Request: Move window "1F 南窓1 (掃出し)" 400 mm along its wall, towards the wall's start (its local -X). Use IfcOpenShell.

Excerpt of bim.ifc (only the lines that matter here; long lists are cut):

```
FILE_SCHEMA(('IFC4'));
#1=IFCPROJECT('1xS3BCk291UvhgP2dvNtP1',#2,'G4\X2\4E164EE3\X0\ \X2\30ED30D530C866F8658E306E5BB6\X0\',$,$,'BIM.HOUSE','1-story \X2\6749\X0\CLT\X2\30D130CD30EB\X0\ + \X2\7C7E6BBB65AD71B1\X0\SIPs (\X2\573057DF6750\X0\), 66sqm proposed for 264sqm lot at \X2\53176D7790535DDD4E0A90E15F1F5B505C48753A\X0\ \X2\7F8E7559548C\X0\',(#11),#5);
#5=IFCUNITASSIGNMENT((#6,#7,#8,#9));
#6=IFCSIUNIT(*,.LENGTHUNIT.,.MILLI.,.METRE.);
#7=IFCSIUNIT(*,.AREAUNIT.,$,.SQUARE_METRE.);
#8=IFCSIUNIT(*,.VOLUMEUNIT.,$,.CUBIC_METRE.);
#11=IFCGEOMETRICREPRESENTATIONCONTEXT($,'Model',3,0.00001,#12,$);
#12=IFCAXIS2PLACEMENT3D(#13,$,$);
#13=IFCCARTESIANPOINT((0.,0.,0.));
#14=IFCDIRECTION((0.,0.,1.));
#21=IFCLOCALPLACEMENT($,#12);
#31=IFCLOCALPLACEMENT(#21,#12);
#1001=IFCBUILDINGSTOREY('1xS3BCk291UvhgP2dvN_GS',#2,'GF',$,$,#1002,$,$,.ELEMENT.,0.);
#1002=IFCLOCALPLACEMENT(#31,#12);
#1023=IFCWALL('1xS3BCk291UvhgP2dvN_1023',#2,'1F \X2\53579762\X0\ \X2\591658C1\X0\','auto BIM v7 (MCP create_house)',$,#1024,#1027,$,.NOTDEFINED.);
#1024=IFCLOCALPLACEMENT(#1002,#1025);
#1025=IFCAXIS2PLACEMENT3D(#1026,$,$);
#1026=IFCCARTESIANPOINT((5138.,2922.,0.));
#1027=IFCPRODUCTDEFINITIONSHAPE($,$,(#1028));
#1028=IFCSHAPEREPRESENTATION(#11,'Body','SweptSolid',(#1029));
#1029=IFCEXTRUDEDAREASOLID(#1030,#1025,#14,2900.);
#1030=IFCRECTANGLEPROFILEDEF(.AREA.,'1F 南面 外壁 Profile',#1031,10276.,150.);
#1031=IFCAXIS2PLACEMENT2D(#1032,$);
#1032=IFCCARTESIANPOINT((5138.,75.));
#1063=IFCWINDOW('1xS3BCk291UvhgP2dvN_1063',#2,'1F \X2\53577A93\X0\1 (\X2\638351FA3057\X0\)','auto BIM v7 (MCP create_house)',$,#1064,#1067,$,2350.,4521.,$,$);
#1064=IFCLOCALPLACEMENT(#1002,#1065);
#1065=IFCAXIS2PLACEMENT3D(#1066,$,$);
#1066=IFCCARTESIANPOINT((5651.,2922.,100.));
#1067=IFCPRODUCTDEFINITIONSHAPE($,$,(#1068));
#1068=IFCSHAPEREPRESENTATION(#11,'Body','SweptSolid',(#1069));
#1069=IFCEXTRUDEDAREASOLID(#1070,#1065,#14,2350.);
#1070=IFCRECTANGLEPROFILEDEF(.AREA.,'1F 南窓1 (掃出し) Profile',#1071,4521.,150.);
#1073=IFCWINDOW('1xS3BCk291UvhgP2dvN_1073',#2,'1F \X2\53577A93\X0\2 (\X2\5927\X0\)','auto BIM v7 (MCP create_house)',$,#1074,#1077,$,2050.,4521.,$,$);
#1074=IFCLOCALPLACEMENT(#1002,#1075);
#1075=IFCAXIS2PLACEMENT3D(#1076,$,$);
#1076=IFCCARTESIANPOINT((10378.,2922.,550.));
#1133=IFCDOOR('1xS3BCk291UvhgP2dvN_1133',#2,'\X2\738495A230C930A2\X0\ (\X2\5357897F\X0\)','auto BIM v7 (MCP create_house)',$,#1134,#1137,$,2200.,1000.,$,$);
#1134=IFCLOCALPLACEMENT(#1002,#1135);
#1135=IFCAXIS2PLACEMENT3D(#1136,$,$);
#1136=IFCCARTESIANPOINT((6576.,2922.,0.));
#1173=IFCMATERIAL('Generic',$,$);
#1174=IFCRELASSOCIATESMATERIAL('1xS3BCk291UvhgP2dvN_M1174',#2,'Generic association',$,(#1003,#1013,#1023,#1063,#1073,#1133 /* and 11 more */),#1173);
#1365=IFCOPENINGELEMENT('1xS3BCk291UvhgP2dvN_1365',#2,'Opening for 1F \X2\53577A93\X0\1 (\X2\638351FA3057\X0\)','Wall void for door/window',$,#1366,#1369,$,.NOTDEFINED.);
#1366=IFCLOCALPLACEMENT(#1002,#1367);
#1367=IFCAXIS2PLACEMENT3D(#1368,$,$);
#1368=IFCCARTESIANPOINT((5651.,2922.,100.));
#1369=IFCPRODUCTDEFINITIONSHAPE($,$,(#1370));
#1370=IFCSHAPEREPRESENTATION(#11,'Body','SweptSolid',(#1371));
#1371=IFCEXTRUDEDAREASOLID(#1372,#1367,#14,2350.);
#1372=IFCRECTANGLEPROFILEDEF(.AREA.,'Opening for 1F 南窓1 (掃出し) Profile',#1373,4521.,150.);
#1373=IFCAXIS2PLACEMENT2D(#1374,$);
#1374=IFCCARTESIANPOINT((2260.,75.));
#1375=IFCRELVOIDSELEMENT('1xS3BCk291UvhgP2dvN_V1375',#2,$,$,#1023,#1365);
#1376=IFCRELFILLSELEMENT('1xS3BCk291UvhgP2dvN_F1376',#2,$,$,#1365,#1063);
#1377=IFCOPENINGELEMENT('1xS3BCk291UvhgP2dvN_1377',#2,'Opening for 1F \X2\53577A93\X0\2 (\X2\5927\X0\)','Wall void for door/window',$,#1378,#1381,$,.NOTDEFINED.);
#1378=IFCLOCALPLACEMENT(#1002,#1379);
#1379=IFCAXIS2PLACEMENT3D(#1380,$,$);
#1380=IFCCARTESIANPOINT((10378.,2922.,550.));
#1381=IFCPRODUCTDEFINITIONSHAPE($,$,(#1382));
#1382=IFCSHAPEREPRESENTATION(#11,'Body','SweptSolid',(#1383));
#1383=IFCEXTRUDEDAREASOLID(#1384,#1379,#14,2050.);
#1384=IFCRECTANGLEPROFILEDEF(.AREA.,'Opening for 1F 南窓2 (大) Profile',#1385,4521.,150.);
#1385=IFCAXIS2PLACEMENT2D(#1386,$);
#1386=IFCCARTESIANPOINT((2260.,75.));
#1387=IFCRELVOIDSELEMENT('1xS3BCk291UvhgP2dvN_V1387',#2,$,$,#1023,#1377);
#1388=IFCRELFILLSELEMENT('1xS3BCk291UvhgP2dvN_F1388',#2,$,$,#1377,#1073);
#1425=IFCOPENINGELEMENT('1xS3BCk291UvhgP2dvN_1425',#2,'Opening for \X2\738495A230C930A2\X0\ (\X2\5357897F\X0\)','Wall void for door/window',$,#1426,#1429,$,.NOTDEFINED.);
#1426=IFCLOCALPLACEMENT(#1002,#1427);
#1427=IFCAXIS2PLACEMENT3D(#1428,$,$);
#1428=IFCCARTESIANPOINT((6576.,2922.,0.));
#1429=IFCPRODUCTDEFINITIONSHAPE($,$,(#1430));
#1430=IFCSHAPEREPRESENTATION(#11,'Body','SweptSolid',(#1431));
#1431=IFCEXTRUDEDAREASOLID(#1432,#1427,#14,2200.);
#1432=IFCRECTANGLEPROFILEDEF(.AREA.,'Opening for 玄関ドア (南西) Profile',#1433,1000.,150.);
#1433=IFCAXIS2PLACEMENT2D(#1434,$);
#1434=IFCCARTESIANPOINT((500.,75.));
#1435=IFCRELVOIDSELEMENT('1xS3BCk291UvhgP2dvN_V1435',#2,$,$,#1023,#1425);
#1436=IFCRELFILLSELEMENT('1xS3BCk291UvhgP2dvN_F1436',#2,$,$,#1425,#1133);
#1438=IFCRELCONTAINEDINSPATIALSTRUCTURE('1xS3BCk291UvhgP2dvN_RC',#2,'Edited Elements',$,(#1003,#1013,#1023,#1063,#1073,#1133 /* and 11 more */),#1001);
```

```python
import ifcopenshell
import ifcopenshell.api.geometry
import ifcopenshell.util.placement
import ifcopenshell.util.unit

model = ifcopenshell.open("bim.ifc")
unit_scale = ifcopenshell.util.unit.calculate_unit_scale(model)

window = model.by_id(1063)
opening = window.FillsVoids[0].RelatingOpeningElement
wall = opening.VoidsElements[0].RelatingBuildingElement

wall_matrix = ifcopenshell.util.placement.get_local_placement(wall.ObjectPlacement)
shift = wall_matrix[:3, 0] * -0.4 / unit_scale
before = ifcopenshell.util.placement.get_local_placement(window.ObjectPlacement)[:3, 3].copy()

# The window is not placed relative to its opening, so move both.
for product in (opening, window):
    matrix = ifcopenshell.util.placement.get_local_placement(product.ObjectPlacement)
    matrix[:3, 3] += shift
    ifcopenshell.api.geometry.edit_object_placement(model, product=product, matrix=matrix, is_si=False)

after = ifcopenshell.util.placement.get_local_placement(window.ObjectPlacement)[:3, 3]
print("window moved by", (after - before).round(3) + 0.0)

model.write("bim_updated.ifc")
```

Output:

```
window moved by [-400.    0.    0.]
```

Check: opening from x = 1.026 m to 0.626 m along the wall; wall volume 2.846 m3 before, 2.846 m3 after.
